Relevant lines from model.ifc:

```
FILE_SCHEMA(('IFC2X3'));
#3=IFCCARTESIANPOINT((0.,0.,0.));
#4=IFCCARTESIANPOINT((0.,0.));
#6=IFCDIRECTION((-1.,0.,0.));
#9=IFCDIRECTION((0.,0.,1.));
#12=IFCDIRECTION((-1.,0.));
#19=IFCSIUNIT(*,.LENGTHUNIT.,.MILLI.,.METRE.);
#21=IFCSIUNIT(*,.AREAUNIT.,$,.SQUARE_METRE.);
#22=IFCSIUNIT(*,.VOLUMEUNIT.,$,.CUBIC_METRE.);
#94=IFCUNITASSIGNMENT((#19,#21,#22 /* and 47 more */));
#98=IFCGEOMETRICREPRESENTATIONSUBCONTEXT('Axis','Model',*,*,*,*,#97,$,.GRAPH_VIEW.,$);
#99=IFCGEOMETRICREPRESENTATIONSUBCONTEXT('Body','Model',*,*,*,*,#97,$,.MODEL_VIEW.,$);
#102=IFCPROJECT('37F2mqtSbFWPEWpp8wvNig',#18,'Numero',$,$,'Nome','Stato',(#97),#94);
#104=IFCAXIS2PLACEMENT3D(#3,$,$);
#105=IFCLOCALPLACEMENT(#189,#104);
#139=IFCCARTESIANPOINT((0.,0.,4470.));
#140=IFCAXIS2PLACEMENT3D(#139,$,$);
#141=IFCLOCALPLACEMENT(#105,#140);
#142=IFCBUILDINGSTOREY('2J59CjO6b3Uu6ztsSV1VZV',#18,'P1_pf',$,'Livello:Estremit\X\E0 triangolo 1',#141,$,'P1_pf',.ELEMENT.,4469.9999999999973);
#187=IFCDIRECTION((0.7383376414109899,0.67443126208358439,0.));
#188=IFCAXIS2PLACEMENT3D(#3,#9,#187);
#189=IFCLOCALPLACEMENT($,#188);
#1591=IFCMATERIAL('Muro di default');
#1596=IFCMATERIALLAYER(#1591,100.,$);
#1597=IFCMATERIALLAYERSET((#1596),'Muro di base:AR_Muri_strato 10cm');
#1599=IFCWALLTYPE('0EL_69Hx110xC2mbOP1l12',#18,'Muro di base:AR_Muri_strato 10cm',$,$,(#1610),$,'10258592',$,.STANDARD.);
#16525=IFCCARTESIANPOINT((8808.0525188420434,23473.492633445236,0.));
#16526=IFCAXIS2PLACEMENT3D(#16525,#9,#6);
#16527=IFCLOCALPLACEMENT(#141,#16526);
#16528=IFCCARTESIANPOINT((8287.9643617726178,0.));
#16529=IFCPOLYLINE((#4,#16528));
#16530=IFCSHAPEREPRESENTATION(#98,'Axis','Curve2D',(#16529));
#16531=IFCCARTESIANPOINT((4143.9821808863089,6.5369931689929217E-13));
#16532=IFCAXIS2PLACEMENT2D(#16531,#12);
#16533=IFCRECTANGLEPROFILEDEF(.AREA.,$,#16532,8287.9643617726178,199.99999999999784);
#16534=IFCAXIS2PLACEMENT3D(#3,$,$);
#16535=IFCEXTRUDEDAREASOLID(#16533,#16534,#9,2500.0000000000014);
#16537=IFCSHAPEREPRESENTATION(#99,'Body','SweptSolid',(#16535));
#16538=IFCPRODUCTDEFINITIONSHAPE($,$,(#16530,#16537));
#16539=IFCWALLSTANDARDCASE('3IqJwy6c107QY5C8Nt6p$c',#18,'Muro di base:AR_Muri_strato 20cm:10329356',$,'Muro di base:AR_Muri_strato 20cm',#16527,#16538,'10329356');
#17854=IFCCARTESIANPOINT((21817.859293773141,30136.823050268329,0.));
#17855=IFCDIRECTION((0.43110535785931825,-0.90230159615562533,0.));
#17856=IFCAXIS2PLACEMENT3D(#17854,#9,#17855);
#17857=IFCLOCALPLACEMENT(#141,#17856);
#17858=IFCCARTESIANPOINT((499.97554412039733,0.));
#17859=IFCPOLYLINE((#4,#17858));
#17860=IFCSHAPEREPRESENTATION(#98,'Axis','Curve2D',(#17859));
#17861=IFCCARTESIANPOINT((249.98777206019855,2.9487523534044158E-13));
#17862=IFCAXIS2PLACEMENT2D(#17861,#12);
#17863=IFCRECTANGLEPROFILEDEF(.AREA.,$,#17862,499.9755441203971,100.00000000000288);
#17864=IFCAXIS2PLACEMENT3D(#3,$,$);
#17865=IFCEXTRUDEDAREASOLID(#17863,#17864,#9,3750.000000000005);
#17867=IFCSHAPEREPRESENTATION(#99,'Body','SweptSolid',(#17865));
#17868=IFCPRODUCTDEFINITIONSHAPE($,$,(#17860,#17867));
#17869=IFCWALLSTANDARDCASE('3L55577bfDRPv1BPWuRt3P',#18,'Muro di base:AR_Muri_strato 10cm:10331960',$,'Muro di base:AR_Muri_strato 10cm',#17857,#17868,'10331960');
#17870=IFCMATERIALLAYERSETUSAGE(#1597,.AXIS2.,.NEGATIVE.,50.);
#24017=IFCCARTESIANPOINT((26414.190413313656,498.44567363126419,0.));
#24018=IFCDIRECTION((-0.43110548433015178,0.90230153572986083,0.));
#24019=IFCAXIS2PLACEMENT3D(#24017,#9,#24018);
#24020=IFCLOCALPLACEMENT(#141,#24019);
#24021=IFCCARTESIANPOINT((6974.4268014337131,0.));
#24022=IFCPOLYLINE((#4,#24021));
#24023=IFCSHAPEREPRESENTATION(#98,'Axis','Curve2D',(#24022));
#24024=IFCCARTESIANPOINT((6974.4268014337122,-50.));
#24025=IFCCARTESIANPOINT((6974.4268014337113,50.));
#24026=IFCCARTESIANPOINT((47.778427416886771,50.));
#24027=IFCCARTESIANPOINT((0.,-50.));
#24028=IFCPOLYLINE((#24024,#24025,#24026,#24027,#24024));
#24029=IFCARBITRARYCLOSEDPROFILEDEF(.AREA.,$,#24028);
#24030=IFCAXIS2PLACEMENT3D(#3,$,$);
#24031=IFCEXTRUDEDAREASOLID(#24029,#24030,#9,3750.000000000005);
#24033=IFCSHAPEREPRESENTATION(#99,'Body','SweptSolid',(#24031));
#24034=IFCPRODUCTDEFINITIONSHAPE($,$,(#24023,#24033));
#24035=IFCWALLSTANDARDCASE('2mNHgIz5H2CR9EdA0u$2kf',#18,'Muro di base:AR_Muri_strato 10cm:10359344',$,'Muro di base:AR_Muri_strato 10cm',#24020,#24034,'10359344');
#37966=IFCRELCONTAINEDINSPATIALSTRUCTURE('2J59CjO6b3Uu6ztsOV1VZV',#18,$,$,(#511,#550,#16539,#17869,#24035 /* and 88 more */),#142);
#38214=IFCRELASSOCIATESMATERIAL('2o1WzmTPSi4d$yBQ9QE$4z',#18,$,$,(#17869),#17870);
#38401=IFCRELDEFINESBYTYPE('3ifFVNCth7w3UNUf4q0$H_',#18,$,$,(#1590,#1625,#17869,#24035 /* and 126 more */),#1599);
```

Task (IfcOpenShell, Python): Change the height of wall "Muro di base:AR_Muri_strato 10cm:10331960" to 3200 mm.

```python
import ifcopenshell
import ifcopenshell.geom
import ifcopenshell.util.representation
import ifcopenshell.util.shape
import ifcopenshell.util.unit

model = ifcopenshell.open("model.ifc")
unit_scale = ifcopenshell.util.unit.calculate_unit_scale(model)
settings = ifcopenshell.geom.settings()


def volume(element):
    """Net volume in cubic metres, openings subtracted."""
    shape = ifcopenshell.geom.create_shape(settings, element)
    return ifcopenshell.util.shape.get_volume(shape.geometry)


wall = model.by_id(17869)
before = volume(wall)

body = ifcopenshell.util.representation.get_representation(wall, "Model", "Body")
solid = body.Items[0]
old_height = solid.Depth
solid.Depth = 3.2 / unit_scale
after = volume(wall)

print(f"height {old_height:g} -> {solid.Depth:g}, volume {before:.3f} -> {after:.3f} m3")

model.write("model_edited.ifc")
```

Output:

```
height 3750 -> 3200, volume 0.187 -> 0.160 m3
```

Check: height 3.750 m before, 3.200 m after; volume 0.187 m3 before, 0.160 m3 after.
